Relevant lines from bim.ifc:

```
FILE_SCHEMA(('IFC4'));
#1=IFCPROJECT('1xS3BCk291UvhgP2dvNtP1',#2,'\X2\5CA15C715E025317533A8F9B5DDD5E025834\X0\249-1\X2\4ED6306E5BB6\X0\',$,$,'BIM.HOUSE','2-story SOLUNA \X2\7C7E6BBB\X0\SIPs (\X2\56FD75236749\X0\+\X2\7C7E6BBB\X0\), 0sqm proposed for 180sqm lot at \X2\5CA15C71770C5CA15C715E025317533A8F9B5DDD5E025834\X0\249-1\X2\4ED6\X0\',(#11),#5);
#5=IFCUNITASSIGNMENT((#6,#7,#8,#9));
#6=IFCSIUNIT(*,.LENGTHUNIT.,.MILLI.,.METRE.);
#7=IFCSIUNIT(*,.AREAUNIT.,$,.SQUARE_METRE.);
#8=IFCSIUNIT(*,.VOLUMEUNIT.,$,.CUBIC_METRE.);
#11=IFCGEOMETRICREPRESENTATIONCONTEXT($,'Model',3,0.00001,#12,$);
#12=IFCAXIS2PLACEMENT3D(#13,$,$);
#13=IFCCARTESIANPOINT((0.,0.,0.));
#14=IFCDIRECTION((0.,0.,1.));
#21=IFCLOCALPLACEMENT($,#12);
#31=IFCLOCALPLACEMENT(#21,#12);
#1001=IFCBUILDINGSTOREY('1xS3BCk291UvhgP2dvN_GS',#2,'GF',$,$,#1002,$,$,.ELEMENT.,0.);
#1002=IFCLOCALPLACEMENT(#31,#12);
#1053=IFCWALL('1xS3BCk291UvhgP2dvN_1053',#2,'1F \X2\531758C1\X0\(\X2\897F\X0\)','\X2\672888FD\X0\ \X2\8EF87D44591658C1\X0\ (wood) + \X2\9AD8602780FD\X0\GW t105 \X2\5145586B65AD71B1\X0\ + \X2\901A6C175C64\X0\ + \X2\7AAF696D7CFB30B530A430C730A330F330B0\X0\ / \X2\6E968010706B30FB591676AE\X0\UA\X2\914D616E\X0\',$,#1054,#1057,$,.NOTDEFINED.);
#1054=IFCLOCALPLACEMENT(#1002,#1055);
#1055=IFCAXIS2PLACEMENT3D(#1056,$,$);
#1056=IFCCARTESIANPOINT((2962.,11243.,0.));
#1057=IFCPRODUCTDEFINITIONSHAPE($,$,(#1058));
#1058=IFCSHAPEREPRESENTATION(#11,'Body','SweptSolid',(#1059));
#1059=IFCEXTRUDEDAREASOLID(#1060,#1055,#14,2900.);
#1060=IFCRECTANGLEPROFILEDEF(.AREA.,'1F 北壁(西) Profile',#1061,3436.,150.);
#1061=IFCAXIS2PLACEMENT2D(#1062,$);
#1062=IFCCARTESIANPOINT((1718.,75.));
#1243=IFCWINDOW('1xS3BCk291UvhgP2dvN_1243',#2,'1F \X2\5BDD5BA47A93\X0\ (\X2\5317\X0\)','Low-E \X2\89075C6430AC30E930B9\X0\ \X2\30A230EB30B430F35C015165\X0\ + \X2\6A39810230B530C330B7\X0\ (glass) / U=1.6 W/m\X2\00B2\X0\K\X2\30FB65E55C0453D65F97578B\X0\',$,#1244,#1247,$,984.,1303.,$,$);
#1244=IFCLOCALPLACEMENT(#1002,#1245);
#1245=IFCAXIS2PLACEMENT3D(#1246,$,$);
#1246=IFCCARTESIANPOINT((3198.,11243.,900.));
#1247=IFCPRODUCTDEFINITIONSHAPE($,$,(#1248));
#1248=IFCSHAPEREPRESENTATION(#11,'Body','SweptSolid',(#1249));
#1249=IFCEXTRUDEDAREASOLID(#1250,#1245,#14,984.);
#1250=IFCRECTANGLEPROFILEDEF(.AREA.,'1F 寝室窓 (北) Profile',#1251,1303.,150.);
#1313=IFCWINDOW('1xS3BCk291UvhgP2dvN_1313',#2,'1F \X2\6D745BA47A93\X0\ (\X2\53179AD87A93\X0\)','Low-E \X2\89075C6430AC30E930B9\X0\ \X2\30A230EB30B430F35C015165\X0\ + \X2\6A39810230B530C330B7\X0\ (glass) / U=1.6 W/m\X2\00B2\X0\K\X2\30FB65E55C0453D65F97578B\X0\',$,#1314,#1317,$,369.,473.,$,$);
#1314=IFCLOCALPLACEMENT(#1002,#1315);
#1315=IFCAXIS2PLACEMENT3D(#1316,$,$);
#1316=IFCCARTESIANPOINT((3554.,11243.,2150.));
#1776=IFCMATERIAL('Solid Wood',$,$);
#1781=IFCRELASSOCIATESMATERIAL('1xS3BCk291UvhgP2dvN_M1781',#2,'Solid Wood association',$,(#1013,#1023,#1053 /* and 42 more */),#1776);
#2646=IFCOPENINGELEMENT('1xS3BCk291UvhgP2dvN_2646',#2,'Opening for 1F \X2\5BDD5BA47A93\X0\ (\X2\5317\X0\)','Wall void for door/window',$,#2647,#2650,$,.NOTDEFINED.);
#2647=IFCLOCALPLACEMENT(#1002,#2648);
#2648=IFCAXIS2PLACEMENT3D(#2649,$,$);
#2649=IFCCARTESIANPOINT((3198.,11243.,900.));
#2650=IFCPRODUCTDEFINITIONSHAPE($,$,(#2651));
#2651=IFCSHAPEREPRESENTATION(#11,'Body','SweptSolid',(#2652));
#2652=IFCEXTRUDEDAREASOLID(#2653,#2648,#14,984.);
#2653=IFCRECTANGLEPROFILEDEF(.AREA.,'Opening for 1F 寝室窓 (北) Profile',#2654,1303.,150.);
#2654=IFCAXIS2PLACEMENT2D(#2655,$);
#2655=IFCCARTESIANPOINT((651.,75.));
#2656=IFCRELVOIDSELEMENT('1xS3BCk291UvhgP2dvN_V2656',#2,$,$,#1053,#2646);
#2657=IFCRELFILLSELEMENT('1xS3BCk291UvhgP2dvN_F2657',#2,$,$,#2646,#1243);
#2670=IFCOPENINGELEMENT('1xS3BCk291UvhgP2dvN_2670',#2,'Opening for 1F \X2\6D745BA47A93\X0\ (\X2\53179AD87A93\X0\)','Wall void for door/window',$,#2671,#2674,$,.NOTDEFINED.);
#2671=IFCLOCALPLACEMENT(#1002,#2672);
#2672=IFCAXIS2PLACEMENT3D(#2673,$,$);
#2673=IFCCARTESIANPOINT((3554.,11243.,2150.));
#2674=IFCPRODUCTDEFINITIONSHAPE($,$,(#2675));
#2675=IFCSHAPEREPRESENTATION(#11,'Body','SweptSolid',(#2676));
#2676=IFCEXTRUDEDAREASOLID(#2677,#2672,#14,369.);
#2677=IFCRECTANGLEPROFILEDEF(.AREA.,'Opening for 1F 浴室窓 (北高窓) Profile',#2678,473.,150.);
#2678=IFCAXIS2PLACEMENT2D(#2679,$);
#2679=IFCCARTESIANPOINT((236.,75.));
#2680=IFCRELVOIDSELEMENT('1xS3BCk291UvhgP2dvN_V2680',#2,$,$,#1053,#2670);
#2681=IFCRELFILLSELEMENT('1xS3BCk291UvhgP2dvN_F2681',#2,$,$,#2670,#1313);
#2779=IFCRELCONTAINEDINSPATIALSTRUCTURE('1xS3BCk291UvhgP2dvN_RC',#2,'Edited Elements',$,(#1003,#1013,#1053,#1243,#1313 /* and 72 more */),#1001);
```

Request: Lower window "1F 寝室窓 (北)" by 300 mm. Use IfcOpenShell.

```python
import numpy as np
import ifcopenshell
import ifcopenshell.api.geometry
import ifcopenshell.util.placement
import ifcopenshell.util.unit

model = ifcopenshell.open("bim.ifc")
unit_scale = ifcopenshell.util.unit.calculate_unit_scale(model)

window = model.by_guid("1xS3BCk291UvhgP2dvN_1243")
opening = window.FillsVoids[0].RelatingOpeningElement
dz = -0.3 / unit_scale

shift = np.array([0.0, 0.0, dz])
# The window is not placed relative to its opening, so move both.
for product in (opening, window):
    matrix = ifcopenshell.util.placement.get_local_placement(product.ObjectPlacement)
    matrix[:3, 3] += shift
    ifcopenshell.api.geometry.edit_object_placement(model, product=product, matrix=matrix, is_si=False)

print(f"moved by {dz * unit_scale:+.3f} m")

model.write("bim_updated.ifc")
```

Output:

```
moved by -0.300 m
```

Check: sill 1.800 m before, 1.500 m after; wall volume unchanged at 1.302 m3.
